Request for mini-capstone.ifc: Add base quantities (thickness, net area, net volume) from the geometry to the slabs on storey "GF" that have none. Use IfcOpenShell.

First a look at what the model holds.

```python
import ifcopenshell
import ifcopenshell.util.element
import ifcopenshell.util.unit

model = ifcopenshell.open("mini-capstone.ifc")
print(model.schema)
for unit_type in ("LENGTHUNIT", "AREAUNIT", "VOLUMEUNIT"):
    print(unit_type, ifcopenshell.util.unit.calculate_unit_scale(model, unit_type))
storey = next(s for s in model.by_type("IfcBuildingStorey") if s.Name == "GF")
slabs = [e for e in ifcopenshell.util.element.get_decomposition(storey) if e.is_a("IfcSlab")]
for e in sorted(slabs, key=lambda e: e.id()):
    print(e.id(), e.is_a(), e.Name, list(ifcopenshell.util.element.get_psets(e, qtos_only=True)), sep=" | ")
```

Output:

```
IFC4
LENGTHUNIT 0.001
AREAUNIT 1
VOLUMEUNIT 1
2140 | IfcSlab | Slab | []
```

```python
import ifcopenshell
import ifcopenshell.api.pset
import ifcopenshell.geom
import ifcopenshell.util.element
import ifcopenshell.util.shape
import ifcopenshell.util.unit

model = ifcopenshell.open("mini-capstone.ifc")
unit_scale = ifcopenshell.util.unit.calculate_unit_scale(model)
area_scale = ifcopenshell.util.unit.calculate_unit_scale(model, "AREAUNIT")
volume_scale = ifcopenshell.util.unit.calculate_unit_scale(model, "VOLUMEUNIT")
settings = ifcopenshell.geom.settings()

storey = next(s for s in model.by_type("IfcBuildingStorey") if s.Name == "GF")
slabs = [e for e in ifcopenshell.util.element.get_decomposition(storey) if e.is_a("IfcSlab")]

for e in sorted(slabs, key=lambda e: e.id()):
    if ifcopenshell.util.element.get_psets(e, qtos_only=True, should_inherit=False):
        continue
    # Geometry comes back in metres, in the element's own axes.
    shape = ifcopenshell.geom.create_shape(settings, e)
    values = {
        "Width": ifcopenshell.util.shape.get_z(shape.geometry) / unit_scale,
        "NetArea": ifcopenshell.util.shape.get_footprint_area(shape.geometry) / area_scale,
        "NetVolume": ifcopenshell.util.shape.get_volume(shape.geometry) / volume_scale,
    }
    qto = ifcopenshell.api.pset.add_qto(model, product=e, name="Qto_SlabBaseQuantities")
    ifcopenshell.api.pset.edit_qto(model, qto=qto, properties=values)
    print(e.id(), {k: round(v, 3) for k, v in values.items()})

model.write("mini-capstone_rev.ifc")
```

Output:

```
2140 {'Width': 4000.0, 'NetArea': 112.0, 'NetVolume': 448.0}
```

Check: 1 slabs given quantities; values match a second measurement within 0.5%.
